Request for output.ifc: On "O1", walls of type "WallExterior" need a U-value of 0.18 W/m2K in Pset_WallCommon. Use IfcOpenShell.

First a look at what the model holds.

```python
import ifcopenshell
import ifcopenshell.util.element

model = ifcopenshell.open("output.ifc")
print(model.schema)
storey = next(s for s in model.by_type("IfcBuildingStorey") if s.Name == "O1")
walls = [e for e in ifcopenshell.util.element.get_decomposition(storey) if e.is_a("IfcWall")]
seen = {}
for e in walls:
    element_type = ifcopenshell.util.element.get_type(e)
    key = (element_type.Name if element_type != e and element_type else None, ifcopenshell.util.element.get_pset(e, "Pset_WallCommon", "ThermalTransmittance"))
    seen[key] = seen.get(key, 0) + 1
for (name, value), count in sorted(seen.items(), key=str):
    print(count, "x", name, "|", value)
```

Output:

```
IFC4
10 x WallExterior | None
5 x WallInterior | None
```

```python
import ifcopenshell
import ifcopenshell.api.pset
import ifcopenshell.util.element

model = ifcopenshell.open("output.ifc")

storey = next(s for s in model.by_type("IfcBuildingStorey") if s.Name == "O1")
walls = [e for e in ifcopenshell.util.element.get_decomposition(storey) if e.is_a("IfcWall")]

count = 0
for e in walls:
    element_type = ifcopenshell.util.element.get_type(e)
    if element_type in (None, e) or element_type.Name != "WallExterior":
        continue
    # add_pset returns the element's existing set when there is one.
    pset = ifcopenshell.api.pset.add_pset(model, product=e, name="Pset_WallCommon")
    ifcopenshell.api.pset.edit_pset(model, pset=pset, properties={"ThermalTransmittance": 0.18})
    count += 1

print(count, "walls updated")

model.write("output_rev.ifc")
```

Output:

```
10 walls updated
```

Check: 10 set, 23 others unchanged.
